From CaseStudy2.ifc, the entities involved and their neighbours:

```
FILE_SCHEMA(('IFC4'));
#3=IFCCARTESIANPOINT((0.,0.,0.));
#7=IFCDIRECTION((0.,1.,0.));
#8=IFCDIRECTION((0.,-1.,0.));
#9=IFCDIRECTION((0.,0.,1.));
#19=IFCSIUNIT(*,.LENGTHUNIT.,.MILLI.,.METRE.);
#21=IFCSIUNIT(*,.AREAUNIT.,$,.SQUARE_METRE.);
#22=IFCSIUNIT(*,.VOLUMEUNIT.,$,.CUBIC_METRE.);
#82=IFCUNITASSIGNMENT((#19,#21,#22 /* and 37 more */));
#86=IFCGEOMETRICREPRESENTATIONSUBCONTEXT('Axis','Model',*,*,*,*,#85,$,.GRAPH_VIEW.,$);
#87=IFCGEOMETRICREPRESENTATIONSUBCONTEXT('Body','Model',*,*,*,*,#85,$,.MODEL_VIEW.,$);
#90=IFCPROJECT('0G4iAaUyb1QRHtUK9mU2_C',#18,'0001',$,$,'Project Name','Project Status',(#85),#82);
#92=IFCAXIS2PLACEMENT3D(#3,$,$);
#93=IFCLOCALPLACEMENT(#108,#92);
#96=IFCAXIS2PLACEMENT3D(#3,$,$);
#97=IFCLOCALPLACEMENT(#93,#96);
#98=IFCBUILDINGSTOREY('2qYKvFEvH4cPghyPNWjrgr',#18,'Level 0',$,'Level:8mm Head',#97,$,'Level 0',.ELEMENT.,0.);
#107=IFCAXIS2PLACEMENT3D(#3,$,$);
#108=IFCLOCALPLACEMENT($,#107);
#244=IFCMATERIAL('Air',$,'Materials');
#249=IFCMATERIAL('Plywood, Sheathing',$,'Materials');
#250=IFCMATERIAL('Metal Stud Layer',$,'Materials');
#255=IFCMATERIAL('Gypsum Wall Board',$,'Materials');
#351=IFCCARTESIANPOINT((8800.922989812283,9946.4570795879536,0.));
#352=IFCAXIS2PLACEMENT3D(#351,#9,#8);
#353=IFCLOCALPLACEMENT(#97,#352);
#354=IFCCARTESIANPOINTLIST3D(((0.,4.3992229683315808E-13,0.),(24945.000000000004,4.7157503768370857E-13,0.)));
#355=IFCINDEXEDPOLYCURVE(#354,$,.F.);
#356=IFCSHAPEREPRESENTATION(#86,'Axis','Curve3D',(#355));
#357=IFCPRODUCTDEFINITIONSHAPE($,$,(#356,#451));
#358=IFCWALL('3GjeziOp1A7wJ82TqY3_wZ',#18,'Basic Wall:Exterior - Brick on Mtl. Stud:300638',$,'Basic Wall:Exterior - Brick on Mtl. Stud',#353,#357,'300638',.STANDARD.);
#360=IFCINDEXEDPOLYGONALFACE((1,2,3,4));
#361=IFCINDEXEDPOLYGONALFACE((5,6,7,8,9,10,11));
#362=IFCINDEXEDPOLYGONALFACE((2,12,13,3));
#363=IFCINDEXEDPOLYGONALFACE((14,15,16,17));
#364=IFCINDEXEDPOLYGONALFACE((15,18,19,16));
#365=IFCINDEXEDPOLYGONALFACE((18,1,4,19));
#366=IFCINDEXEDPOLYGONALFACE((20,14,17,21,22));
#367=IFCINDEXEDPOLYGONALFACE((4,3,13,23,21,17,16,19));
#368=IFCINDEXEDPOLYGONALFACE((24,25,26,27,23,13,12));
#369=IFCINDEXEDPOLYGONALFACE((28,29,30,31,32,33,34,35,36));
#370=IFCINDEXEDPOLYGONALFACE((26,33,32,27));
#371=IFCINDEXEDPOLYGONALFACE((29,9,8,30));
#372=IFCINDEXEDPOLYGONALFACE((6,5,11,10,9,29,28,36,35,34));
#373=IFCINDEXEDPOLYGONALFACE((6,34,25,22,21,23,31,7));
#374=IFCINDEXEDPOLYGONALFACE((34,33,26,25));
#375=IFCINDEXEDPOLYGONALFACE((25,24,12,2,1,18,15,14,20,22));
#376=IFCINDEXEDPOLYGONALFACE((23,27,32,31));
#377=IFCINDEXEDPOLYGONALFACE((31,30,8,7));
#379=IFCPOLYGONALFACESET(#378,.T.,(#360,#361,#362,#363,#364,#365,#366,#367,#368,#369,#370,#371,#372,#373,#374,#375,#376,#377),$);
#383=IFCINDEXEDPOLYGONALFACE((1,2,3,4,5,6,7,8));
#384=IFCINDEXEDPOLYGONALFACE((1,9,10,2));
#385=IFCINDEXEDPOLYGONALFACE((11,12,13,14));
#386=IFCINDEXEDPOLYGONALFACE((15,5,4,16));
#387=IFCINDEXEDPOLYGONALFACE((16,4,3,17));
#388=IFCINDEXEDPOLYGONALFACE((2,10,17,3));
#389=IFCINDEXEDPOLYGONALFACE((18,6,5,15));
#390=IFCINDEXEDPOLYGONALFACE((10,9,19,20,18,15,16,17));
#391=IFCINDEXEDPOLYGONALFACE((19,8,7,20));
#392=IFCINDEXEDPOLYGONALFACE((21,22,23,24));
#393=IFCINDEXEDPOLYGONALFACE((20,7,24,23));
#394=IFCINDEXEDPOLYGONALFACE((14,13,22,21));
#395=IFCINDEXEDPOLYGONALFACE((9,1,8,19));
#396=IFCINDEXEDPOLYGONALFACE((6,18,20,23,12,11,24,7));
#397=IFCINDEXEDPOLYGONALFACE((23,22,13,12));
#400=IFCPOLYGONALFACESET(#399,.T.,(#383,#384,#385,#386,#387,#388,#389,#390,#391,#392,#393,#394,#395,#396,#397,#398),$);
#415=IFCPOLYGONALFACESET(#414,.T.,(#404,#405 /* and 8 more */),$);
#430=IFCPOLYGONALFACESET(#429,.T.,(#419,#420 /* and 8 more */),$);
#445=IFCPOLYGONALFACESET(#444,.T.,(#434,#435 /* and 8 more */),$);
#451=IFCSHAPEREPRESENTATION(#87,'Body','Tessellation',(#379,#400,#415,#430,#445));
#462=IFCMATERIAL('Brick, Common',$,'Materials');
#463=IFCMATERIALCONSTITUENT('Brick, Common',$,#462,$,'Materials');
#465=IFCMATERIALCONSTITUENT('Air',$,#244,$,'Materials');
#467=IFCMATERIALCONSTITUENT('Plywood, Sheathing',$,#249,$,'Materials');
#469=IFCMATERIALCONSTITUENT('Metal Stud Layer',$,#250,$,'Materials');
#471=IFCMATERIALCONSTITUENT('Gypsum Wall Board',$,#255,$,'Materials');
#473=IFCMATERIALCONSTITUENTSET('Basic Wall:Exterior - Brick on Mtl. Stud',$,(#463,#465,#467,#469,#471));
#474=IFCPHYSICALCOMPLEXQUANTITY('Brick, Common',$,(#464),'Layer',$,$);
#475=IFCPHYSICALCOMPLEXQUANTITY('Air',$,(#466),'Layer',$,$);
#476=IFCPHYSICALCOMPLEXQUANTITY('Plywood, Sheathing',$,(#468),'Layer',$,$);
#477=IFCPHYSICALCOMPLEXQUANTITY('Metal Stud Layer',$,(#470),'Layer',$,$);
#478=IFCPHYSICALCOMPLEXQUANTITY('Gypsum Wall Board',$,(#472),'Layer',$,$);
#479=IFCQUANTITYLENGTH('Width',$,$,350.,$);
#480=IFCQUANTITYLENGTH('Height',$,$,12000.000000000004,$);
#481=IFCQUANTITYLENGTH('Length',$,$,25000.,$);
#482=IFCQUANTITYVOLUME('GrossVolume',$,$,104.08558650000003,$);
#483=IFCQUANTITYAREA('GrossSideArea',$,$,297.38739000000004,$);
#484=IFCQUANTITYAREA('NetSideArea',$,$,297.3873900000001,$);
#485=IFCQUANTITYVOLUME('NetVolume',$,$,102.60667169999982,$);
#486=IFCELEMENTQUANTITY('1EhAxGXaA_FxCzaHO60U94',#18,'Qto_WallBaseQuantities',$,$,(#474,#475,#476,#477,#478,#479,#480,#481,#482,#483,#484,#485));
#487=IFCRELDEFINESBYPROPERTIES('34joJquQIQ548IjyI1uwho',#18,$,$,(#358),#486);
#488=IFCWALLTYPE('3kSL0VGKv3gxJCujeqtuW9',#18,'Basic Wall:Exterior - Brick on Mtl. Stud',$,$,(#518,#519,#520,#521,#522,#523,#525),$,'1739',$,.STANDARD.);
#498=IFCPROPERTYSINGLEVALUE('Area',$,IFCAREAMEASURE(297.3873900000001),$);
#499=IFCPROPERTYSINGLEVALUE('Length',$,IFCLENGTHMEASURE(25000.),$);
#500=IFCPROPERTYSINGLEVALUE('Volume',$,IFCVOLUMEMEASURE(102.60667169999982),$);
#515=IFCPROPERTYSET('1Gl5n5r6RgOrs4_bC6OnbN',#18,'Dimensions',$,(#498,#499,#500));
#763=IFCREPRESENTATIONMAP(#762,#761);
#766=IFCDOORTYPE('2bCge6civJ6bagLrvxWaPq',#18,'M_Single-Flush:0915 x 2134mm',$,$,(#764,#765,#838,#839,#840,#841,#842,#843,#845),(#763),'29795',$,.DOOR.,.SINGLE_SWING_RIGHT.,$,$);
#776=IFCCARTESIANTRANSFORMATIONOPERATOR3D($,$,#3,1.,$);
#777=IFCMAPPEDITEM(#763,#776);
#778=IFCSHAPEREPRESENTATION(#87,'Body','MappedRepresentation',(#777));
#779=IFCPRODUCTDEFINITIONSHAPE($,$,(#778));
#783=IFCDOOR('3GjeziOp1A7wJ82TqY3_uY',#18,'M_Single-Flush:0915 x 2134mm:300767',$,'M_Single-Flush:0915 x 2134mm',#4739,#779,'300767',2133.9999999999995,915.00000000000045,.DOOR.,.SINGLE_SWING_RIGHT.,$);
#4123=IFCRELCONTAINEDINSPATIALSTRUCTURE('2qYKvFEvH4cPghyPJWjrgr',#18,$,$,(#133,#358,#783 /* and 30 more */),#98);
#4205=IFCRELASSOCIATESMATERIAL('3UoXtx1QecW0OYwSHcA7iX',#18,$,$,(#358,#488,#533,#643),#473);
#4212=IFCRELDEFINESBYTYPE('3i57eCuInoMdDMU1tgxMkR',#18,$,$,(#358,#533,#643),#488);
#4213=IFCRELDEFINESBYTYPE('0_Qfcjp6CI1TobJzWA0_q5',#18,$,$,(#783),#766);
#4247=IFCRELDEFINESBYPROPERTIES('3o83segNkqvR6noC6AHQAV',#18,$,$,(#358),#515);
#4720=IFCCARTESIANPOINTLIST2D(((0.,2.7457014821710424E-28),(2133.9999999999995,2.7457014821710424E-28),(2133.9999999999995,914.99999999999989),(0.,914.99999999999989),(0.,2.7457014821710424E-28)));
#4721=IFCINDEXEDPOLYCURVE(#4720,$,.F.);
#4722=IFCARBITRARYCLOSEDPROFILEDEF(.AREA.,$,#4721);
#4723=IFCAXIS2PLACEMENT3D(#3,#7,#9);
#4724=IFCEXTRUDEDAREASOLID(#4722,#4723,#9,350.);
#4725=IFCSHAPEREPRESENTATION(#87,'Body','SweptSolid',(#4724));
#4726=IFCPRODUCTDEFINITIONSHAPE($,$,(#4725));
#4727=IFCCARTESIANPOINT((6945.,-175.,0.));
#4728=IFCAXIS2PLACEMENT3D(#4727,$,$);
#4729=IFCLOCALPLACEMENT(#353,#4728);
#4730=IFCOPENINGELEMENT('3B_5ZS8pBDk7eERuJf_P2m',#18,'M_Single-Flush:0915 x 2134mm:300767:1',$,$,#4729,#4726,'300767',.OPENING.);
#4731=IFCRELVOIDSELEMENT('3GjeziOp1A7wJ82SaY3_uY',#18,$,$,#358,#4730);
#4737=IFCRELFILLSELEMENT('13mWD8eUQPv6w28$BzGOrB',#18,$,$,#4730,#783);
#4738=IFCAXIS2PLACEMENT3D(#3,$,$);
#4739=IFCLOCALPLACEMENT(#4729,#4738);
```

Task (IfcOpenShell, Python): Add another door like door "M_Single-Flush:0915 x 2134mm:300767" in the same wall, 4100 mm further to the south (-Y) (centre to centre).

```python
import ifcopenshell
import ifcopenshell.api.feature
import ifcopenshell.api.geometry
import ifcopenshell.api.pset
import ifcopenshell.api.root
import ifcopenshell.geom
import ifcopenshell.util.element
import ifcopenshell.util.placement
import ifcopenshell.util.shape
import ifcopenshell.util.unit

model = ifcopenshell.open("CaseStudy2.ifc")
area_scale = ifcopenshell.util.unit.calculate_unit_scale(model, "AREAUNIT")
volume_scale = ifcopenshell.util.unit.calculate_unit_scale(model, "VOLUMEUNIT")
settings = ifcopenshell.geom.settings()


def volume(element):
    """Net volume in cubic metres, openings subtracted."""
    shape = ifcopenshell.geom.create_shape(settings, element)
    return ifcopenshell.util.shape.get_volume(shape.geometry)


def reuse_history(source, copy):
    """copy_class also copies each property set's owner history, people and application; keep the originals."""
    for rel in copy.IsDefinedBy:
        if rel.is_a("IfcRelDefinesByProperties") and (history := rel.RelatingPropertyDefinition.OwnerHistory):
            rel.RelatingPropertyDefinition.OwnerHistory = source.OwnerHistory
            ifcopenshell.util.element.remove_deep2(model, history)


door = model.by_guid("3GjeziOp1A7wJ82TqY3_uY")
opening = door.FillsVoids[0].RelatingOpeningElement
wall = opening.VoidsElements[0].RelatingBuildingElement
before = volume(wall)
shift = ifcopenshell.util.placement.get_local_placement(wall.ObjectPlacement)[:3, 0] * 4100.0

# copy_class copies the void relationship, type, container and properties, but no geometry.
new_opening = ifcopenshell.api.root.copy_class(model, product=opening)
new_opening.Representation = ifcopenshell.util.element.copy_deep(
    model, opening.Representation, exclude=["IfcGeometricRepresentationContext", "IfcRepresentationMap"]
)
new_opening.Name = "M_Single-Flush:0915 x 2134mm"
new_opening.Tag = None
reuse_history(opening, new_opening)
new_door = ifcopenshell.api.root.copy_class(model, product=door)
new_door.Representation = ifcopenshell.util.element.copy_deep(
    model, door.Representation, exclude=["IfcGeometricRepresentationContext", "IfcRepresentationMap"]
)
new_door.Name = "M_Single-Flush:0915 x 2134mm"
new_door.Tag = None
reuse_history(door, new_door)
ifcopenshell.api.feature.add_filling(model, opening=new_opening, element=new_door)

for old, new in ((opening, new_opening), (door, new_door)):
    matrix = ifcopenshell.util.placement.get_local_placement(old.ObjectPlacement)
    matrix[:3, 3] += shift
    ifcopenshell.api.geometry.edit_object_placement(model, product=new, matrix=matrix, is_si=False)

after = volume(wall)
thickness = 0.35  # wall thickness in metres

# Update the wall's stored quantities.
qto = model.by_id(ifcopenshell.util.element.get_pset(wall, "Qto_WallBaseQuantities", should_inherit=False)["id"])
ifcopenshell.api.pset.edit_qto(model, qto=qto, properties={
    "NetSideArea": after / thickness / area_scale,
    "NetVolume": after / volume_scale,
})
pset = model.by_id(ifcopenshell.util.element.get_pset(wall, "Dimensions", should_inherit=False)["id"])
ifcopenshell.api.pset.edit_pset(model, pset=pset, properties={
    "Area": model.create_entity("IfcAreaMeasure", after / thickness / area_scale),
    "Volume": model.create_entity("IfcVolumeMeasure", after / volume_scale),
})

print(f"wall volume {before:.3f} -> {after:.3f} m3")

model.write("CaseStudy2_rev.ifc")
```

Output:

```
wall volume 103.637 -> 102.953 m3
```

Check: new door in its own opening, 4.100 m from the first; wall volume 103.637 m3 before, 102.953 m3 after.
